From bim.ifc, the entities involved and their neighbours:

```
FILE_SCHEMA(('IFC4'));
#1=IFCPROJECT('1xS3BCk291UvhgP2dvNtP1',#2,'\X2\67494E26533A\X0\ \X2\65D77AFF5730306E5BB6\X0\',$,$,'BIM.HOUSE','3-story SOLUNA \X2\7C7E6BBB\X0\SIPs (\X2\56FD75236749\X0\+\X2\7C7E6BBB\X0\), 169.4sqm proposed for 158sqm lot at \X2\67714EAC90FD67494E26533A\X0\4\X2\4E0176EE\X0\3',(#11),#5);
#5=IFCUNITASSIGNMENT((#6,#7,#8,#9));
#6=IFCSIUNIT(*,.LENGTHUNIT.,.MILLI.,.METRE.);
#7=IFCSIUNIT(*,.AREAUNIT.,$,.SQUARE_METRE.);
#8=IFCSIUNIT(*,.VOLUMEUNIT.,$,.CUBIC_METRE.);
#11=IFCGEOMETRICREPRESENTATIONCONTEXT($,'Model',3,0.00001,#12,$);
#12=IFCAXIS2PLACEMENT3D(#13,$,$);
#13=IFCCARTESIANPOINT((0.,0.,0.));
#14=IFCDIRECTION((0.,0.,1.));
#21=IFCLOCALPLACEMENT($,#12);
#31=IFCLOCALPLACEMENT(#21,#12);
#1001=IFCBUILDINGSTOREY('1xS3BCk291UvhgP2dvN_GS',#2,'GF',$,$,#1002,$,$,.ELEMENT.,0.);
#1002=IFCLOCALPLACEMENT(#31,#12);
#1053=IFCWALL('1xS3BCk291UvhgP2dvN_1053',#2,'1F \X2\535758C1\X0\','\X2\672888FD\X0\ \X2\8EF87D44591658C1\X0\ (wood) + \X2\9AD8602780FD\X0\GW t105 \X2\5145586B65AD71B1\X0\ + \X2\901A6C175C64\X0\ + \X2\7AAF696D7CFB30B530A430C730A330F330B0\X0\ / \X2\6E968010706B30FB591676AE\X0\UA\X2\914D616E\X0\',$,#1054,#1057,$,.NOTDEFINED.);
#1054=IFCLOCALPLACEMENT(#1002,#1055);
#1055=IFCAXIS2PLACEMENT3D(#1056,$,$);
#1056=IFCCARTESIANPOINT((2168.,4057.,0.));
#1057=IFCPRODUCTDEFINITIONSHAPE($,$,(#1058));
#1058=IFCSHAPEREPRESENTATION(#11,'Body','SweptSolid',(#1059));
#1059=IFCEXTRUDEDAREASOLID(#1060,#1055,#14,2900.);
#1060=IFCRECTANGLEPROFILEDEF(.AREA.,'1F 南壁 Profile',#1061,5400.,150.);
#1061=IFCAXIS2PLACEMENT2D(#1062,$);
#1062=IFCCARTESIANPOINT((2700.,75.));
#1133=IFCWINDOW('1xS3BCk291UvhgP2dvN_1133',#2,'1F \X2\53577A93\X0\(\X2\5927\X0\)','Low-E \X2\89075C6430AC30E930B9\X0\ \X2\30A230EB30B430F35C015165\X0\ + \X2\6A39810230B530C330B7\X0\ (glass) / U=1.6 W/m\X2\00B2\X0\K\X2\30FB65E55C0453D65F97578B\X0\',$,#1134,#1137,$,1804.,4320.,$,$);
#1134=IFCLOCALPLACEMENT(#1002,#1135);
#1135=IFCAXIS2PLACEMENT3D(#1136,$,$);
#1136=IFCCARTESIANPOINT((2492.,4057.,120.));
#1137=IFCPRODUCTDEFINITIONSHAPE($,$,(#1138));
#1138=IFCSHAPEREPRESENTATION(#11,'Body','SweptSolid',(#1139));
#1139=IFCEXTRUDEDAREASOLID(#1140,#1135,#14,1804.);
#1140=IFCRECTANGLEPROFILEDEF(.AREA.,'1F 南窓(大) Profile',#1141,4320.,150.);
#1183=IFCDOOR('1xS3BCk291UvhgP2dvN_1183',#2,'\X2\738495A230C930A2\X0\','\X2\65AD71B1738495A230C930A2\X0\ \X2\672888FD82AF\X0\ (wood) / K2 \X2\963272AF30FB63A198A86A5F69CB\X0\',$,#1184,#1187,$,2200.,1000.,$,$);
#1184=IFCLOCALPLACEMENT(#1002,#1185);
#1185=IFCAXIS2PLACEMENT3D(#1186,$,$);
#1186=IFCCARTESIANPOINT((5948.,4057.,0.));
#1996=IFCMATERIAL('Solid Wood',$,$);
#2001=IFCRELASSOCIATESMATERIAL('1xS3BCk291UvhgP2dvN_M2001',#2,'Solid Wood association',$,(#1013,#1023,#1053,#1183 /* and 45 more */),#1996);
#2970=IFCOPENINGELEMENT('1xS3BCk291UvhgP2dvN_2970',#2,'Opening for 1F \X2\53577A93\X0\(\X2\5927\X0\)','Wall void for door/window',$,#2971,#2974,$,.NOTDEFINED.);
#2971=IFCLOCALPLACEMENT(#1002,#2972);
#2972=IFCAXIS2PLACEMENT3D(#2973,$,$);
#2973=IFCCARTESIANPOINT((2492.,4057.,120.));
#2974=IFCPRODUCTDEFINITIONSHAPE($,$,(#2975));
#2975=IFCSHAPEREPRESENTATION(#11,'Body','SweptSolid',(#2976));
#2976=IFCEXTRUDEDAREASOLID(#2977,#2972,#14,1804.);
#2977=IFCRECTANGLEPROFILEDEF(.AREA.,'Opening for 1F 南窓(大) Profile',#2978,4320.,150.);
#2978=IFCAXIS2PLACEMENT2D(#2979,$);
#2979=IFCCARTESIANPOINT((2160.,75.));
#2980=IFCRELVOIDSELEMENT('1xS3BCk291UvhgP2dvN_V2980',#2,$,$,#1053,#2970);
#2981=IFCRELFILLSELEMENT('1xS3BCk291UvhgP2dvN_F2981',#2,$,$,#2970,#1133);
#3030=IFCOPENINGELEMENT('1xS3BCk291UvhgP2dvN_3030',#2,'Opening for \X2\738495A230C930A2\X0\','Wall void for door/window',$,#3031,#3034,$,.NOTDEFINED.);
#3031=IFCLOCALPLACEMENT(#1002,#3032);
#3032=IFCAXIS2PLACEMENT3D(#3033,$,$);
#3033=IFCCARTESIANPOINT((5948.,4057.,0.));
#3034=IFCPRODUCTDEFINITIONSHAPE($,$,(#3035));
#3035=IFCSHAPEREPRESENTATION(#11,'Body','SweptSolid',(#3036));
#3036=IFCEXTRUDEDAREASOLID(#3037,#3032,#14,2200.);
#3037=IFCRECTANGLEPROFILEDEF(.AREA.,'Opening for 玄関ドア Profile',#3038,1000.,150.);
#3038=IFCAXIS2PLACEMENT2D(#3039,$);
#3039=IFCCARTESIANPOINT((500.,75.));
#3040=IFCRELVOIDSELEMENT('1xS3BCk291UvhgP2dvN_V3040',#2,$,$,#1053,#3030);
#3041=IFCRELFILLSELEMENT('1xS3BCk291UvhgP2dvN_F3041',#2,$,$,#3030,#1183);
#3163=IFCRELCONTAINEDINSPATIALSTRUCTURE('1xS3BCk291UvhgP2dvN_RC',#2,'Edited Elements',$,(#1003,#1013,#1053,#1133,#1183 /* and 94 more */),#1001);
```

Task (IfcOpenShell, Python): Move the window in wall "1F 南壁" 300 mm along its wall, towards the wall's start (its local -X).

```python
import ifcopenshell
import ifcopenshell.api.geometry
import ifcopenshell.util.placement

model = ifcopenshell.open("bim.ifc")

window = model.by_guid("1xS3BCk291UvhgP2dvN_1133")
opening = window.FillsVoids[0].RelatingOpeningElement
wall = opening.VoidsElements[0].RelatingBuildingElement

wall_matrix = ifcopenshell.util.placement.get_local_placement(wall.ObjectPlacement)
shift = wall_matrix[:3, 0] * -300.0
before = ifcopenshell.util.placement.get_local_placement(window.ObjectPlacement)[:3, 3].copy()

# The window is not placed relative to its opening, so move both.
for product in (opening, window):
    matrix = ifcopenshell.util.placement.get_local_placement(product.ObjectPlacement)
    matrix[:3, 3] += shift
    ifcopenshell.api.geometry.edit_object_placement(model, product=product, matrix=matrix, is_si=False)

after = ifcopenshell.util.placement.get_local_placement(window.ObjectPlacement)[:3, 3]
print("window moved by", (after - before).round(3) + 0.0)

model.write("bim_rev.ifc")
```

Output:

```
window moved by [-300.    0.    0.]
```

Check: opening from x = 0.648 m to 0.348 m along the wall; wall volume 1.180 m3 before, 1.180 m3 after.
